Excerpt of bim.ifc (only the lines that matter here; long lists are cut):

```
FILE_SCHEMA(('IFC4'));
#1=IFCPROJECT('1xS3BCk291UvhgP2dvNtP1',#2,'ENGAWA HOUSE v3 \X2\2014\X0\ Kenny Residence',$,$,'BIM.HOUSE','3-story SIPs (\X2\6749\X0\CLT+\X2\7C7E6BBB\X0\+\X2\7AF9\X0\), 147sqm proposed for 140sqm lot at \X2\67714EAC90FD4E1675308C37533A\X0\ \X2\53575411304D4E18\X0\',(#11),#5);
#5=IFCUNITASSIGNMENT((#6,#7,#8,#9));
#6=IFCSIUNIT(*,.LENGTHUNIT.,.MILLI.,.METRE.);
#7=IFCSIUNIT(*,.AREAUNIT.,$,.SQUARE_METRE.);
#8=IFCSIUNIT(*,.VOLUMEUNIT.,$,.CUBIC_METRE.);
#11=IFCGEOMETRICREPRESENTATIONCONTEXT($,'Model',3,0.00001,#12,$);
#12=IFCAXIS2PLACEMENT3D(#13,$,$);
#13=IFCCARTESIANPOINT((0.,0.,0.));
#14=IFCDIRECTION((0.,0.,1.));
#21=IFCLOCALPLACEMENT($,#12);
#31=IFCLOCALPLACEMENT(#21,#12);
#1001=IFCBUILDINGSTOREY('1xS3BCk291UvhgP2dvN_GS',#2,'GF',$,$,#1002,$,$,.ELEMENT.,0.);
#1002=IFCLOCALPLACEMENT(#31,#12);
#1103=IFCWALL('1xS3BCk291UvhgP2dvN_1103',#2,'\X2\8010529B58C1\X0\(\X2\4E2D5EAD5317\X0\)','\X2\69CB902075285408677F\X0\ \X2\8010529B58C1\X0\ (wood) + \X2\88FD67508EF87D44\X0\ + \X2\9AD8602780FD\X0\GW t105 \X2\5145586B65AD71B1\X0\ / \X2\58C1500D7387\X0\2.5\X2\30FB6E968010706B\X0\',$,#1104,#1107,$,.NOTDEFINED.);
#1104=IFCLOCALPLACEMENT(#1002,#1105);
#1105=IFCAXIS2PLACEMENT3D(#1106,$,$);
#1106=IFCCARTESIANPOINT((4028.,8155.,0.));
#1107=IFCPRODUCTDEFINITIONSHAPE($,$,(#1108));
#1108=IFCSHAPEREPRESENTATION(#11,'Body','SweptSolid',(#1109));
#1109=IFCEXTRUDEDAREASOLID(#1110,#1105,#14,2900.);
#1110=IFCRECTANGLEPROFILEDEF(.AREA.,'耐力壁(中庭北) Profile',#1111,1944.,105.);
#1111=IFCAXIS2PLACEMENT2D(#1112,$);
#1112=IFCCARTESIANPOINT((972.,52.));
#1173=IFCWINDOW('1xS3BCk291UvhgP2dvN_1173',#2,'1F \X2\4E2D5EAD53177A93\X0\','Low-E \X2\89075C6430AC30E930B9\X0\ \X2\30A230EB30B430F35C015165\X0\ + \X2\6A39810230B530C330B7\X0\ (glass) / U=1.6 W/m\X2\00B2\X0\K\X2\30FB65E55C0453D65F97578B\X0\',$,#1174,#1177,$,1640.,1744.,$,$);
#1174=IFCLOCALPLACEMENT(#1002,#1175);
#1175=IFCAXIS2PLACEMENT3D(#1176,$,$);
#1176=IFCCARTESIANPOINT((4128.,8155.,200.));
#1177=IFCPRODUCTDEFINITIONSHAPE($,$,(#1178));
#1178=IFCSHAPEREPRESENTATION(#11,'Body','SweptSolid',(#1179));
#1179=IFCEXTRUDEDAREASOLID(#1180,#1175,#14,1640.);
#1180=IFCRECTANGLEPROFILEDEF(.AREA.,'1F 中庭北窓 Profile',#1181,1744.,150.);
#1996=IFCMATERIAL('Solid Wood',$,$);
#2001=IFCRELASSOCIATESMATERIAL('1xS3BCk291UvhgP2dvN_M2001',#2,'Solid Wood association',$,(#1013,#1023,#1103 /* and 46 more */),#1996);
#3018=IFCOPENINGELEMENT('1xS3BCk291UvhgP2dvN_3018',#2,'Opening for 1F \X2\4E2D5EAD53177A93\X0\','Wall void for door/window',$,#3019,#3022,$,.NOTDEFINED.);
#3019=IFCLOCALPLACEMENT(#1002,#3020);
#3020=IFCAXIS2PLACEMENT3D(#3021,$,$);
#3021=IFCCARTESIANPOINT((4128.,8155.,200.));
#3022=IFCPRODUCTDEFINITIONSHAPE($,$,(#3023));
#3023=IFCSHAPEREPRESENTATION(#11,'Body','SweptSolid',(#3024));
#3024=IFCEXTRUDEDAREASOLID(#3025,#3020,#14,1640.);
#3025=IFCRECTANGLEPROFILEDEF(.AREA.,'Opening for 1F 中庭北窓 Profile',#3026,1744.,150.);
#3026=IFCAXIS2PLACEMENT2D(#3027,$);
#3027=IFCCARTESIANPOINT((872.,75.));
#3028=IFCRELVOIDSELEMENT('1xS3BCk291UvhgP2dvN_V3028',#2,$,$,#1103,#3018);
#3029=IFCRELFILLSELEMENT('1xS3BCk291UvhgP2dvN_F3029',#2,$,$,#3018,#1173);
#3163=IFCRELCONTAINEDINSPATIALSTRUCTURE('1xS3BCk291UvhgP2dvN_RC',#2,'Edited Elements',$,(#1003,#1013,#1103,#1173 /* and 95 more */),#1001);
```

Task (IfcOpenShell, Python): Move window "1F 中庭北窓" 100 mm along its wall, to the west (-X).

```python
import ifcopenshell
import ifcopenshell.api.geometry
import ifcopenshell.util.placement
import ifcopenshell.util.unit

model = ifcopenshell.open("bim.ifc")
unit_scale = ifcopenshell.util.unit.calculate_unit_scale(model)

window = model.by_guid("1xS3BCk291UvhgP2dvN_1173")
opening = window.FillsVoids[0].RelatingOpeningElement
wall = opening.VoidsElements[0].RelatingBuildingElement

wall_matrix = ifcopenshell.util.placement.get_local_placement(wall.ObjectPlacement)
shift = wall_matrix[:3, 0] * -0.1 / unit_scale
before = ifcopenshell.util.placement.get_local_placement(window.ObjectPlacement)[:3, 3].copy()

# The window is not placed relative to its opening, so move both.
for product in (opening, window):
    matrix = ifcopenshell.util.placement.get_local_placement(product.ObjectPlacement)
    matrix[:3, 3] += shift
    ifcopenshell.api.geometry.edit_object_placement(model, product=product, matrix=matrix, is_si=False)

after = ifcopenshell.util.placement.get_local_placement(window.ObjectPlacement)[:3, 3]
print("window moved by", (after - before).round(3) + 0.0)

model.write("bim_rev.ifc")
```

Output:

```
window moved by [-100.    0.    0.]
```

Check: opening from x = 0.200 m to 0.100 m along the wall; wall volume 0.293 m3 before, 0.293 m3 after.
